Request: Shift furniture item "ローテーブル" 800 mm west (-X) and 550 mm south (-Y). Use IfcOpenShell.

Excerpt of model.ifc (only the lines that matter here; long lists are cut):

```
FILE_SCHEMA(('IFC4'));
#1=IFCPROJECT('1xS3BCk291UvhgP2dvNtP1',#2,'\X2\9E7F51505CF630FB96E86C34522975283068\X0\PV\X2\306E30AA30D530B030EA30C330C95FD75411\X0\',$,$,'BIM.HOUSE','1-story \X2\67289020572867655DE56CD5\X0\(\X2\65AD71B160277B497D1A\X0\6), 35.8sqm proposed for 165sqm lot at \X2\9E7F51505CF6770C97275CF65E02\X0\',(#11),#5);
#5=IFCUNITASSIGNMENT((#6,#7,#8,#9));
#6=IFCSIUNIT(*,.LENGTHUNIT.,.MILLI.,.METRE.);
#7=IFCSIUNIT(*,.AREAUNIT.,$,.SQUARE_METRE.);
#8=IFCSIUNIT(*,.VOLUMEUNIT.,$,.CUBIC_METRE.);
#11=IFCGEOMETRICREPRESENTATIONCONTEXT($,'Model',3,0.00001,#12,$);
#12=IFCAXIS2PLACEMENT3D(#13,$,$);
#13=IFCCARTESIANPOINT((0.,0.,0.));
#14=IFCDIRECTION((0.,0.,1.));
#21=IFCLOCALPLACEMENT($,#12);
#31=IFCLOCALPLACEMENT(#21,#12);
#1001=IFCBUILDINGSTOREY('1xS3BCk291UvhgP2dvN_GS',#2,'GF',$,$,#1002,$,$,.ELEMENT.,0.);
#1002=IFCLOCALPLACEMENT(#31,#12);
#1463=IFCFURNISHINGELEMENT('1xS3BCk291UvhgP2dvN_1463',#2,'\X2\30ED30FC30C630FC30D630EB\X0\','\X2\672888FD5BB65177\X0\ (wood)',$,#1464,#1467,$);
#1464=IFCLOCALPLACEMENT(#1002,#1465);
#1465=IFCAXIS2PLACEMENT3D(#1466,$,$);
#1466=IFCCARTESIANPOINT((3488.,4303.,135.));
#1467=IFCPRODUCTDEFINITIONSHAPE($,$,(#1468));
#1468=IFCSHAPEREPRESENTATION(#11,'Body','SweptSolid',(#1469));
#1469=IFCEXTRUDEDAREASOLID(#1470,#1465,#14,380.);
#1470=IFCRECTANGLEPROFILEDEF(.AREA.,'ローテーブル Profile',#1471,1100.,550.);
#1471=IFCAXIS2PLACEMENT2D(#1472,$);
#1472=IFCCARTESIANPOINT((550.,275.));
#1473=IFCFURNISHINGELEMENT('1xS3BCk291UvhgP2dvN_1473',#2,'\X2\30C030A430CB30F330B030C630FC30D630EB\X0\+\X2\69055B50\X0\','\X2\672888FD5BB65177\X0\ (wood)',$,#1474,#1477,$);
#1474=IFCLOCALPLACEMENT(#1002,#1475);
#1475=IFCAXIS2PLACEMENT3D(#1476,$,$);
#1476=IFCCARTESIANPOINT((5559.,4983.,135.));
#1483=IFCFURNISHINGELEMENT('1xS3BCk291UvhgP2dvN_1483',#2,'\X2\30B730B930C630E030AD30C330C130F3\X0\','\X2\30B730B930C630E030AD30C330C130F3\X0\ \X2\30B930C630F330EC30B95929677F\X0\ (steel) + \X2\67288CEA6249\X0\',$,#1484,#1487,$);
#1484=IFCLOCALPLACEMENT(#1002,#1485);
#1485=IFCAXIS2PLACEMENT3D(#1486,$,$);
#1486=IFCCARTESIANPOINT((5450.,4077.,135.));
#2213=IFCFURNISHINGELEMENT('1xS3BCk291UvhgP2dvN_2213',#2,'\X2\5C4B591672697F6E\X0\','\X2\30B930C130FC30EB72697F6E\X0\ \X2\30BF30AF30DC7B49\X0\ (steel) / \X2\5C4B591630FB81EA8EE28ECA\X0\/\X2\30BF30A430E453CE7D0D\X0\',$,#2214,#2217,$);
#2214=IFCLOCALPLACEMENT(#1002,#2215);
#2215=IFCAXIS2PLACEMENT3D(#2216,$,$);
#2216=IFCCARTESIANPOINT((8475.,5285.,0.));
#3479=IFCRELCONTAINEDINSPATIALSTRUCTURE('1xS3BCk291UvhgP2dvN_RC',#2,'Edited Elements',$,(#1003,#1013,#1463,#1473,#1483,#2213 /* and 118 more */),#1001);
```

```python
import ifcopenshell
import ifcopenshell.api.geometry
import ifcopenshell.util.placement
import ifcopenshell.util.unit

model = ifcopenshell.open("model.ifc")
unit_scale = ifcopenshell.util.unit.calculate_unit_scale(model)

item = model.by_guid("1xS3BCk291UvhgP2dvN_1463")
matrix = ifcopenshell.util.placement.get_local_placement(item.ObjectPlacement)
matrix[0, 3] -= 0.8 / unit_scale
matrix[1, 3] -= 0.55 / unit_scale
ifcopenshell.api.geometry.edit_object_placement(model, product=item, matrix=matrix, is_si=False)

print(ifcopenshell.util.placement.get_local_placement(item.ObjectPlacement).round(3) + 0.0)

model.write("model_edited.ifc")
```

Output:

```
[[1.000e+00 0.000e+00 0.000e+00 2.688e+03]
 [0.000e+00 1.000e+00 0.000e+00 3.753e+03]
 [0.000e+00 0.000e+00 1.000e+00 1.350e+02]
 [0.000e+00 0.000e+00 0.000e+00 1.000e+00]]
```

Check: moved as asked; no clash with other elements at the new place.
